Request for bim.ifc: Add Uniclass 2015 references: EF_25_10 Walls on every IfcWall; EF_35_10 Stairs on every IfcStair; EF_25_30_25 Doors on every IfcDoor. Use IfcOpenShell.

First a look at what the model holds.

```python
import ifcopenshell

model = ifcopenshell.open("bim.ifc")
print(model.schema)
print("classifications:", [c.Name for c in model.by_type("IfcClassification")])
for ifc_class in ("IfcDoor", "IfcRoof", "IfcStair", "IfcWall", "IfcWindow"):
    print(ifc_class, len(model.by_type(ifc_class)))
```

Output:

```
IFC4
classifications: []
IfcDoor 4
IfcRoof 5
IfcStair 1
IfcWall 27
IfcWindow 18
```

```python
import ifcopenshell
import ifcopenshell.api.classification

model = ifcopenshell.open("bim.ifc")

system = ifcopenshell.api.classification.add_classification(model, classification="Uniclass 2015")

codes = {
    "IfcWall": ("EF_25_10", "Walls"),
    "IfcStair": ("EF_35_10", "Stairs"),
    "IfcDoor": ("EF_25_30_25", "Doors"),
}
for ifc_class, (code, name) in codes.items():
    products = model.by_type(ifc_class)
    ifcopenshell.api.classification.add_reference(
        model, products=products, classification=system, identification=code, name=name
    )
    print(code, len(products))

model.write("bim_edited.ifc")
```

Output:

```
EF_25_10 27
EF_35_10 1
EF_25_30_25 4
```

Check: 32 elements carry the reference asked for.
